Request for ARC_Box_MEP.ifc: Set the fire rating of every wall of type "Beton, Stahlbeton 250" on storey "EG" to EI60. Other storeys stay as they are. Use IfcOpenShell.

First a look at what the model holds.

```python
import ifcopenshell
import ifcopenshell.util.element

model = ifcopenshell.open("ARC_Box_MEP.ifc")
print(model.schema)
storey = next(s for s in model.by_type("IfcBuildingStorey") if s.Name == "EG")
walls = [e for e in ifcopenshell.util.element.get_decomposition(storey) if e.is_a("IfcWall")]
seen = {}
for e in walls:
    element_type = ifcopenshell.util.element.get_type(e)
    key = (element_type.Name if element_type != e and element_type else None, ifcopenshell.util.element.get_pset(e, "Pset_WallCommon", "FireRating"))
    seen[key] = seen.get(key, 0) + 1
for (name, value), count in sorted(seen.items(), key=str):
    print(count, "x", name, "|", value)
```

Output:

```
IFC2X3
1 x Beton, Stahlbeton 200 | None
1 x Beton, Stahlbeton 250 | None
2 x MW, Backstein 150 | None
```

```python
import ifcopenshell
import ifcopenshell.api.pset
import ifcopenshell.util.element

model = ifcopenshell.open("ARC_Box_MEP.ifc")

storey = next(s for s in model.by_type("IfcBuildingStorey") if s.Name == "EG")
walls = [e for e in ifcopenshell.util.element.get_decomposition(storey) if e.is_a("IfcWall")]

count = 0
for e in walls:
    element_type = ifcopenshell.util.element.get_type(e)
    if element_type in (None, e) or element_type.Name != "Beton, Stahlbeton 250":
        continue
    # add_pset returns the element's existing set when there is one.
    pset = ifcopenshell.api.pset.add_pset(model, product=e, name="Pset_WallCommon")
    ifcopenshell.api.pset.edit_pset(model, pset=pset, properties={"FireRating": "EI60"})
    count += 1

print(count, "walls updated")

model.write("ARC_Box_MEP_edited.ifc")
```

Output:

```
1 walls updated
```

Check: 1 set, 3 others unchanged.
